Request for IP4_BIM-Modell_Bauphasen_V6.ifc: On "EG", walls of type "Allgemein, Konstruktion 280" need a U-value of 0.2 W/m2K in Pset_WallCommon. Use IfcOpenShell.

First a look at what the model holds.

```python
import ifcopenshell
import ifcopenshell.util.element

model = ifcopenshell.open("IP4_BIM-Modell_Bauphasen_V6.ifc")
print(model.schema)
storey = next(s for s in model.by_type("IfcBuildingStorey") if s.Name == "EG")
walls = [e for e in ifcopenshell.util.element.get_decomposition(storey) if e.is_a("IfcWall")]
seen = {}
for e in walls:
    element_type = ifcopenshell.util.element.get_type(e)
    key = (element_type.Name if element_type != e and element_type else None, ifcopenshell.util.element.get_pset(e, "Pset_WallCommon", "ThermalTransmittance"))
    seen[key] = seen.get(key, 0) + 1
for (name, value), count in sorted(seen.items(), key=str):
    print(count, "x", name, "|", value)
```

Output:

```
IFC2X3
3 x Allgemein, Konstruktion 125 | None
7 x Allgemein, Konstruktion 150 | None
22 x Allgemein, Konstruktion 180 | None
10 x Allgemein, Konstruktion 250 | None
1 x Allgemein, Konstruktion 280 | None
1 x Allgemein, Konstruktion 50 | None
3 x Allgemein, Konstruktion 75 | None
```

```python
import ifcopenshell
import ifcopenshell.api.pset
import ifcopenshell.util.element

model = ifcopenshell.open("IP4_BIM-Modell_Bauphasen_V6.ifc")

storey = next(s for s in model.by_type("IfcBuildingStorey") if s.Name == "EG")
walls = [e for e in ifcopenshell.util.element.get_decomposition(storey) if e.is_a("IfcWall")]

count = 0
for e in walls:
    element_type = ifcopenshell.util.element.get_type(e)
    if element_type in (None, e) or element_type.Name != "Allgemein, Konstruktion 280":
        continue
    # add_pset returns the element's existing set when there is one.
    pset = ifcopenshell.api.pset.add_pset(model, product=e, name="Pset_WallCommon")
    ifcopenshell.api.pset.edit_pset(model, pset=pset, properties={"ThermalTransmittance": 0.2})
    count += 1

print(count, "walls updated")

model.write("IP4_BIM-Modell_Bauphasen_V6_v2.ifc")
```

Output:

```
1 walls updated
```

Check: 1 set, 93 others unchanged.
